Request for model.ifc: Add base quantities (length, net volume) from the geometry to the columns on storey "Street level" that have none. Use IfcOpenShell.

First a look at what the model holds.

```python
import ifcopenshell
import ifcopenshell.util.element
import ifcopenshell.util.unit

model = ifcopenshell.open("model.ifc")
print(model.schema)
for unit_type in ("LENGTHUNIT", "AREAUNIT", "VOLUMEUNIT"):
    print(unit_type, ifcopenshell.util.unit.calculate_unit_scale(model, unit_type))
storey = next(s for s in model.by_type("IfcBuildingStorey") if s.Name == "Street level")
columns = [e for e in ifcopenshell.util.element.get_decomposition(storey) if e.is_a("IfcColumn")]
for e in sorted(columns, key=lambda e: e.id()):
    print(e.id(), e.is_a(), e.Name, list(ifcopenshell.util.element.get_psets(e, qtos_only=True)), sep=" | ")
```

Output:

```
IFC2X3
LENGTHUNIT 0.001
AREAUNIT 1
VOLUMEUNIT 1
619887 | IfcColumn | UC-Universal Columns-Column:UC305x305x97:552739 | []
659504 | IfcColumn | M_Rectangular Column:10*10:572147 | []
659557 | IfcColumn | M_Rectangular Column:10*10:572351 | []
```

```python
import ifcopenshell
import ifcopenshell.api.pset
import ifcopenshell.geom
import ifcopenshell.util.element
import ifcopenshell.util.shape
import ifcopenshell.util.unit

model = ifcopenshell.open("model.ifc")
unit_scale = ifcopenshell.util.unit.calculate_unit_scale(model)
volume_scale = ifcopenshell.util.unit.calculate_unit_scale(model, "VOLUMEUNIT")
settings = ifcopenshell.geom.settings()

storey = next(s for s in model.by_type("IfcBuildingStorey") if s.Name == "Street level")
columns = [e for e in ifcopenshell.util.element.get_decomposition(storey) if e.is_a("IfcColumn")]

for e in sorted(columns, key=lambda e: e.id()):
    if ifcopenshell.util.element.get_psets(e, qtos_only=True, should_inherit=False):
        continue
    # Geometry comes back in metres, in the element's own axes.
    shape = ifcopenshell.geom.create_shape(settings, e)
    values = {
        "Length": ifcopenshell.util.shape.get_z(shape.geometry) / unit_scale,
        "NetVolume": ifcopenshell.util.shape.get_volume(shape.geometry) / volume_scale,
    }
    qto = ifcopenshell.api.pset.add_qto(model, product=e, name="BaseQuantities")
    ifcopenshell.api.pset.edit_qto(model, qto=qto, properties=values)
    print(e.id(), {k: round(v, 3) for k, v in values.items()})

model.write("model_rev.ifc")
```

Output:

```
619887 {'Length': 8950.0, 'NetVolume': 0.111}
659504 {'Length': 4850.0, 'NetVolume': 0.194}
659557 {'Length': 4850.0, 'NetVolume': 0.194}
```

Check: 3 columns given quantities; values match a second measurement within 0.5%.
